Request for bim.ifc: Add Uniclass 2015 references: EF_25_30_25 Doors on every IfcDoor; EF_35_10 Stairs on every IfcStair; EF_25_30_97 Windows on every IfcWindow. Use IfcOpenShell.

First a look at what the model holds.

```python
import ifcopenshell

model = ifcopenshell.open("bim.ifc")
print(model.schema)
print("classifications:", [c.Name for c in model.by_type("IfcClassification")])
for ifc_class in ("IfcDoor", "IfcRoof", "IfcStair", "IfcWall", "IfcWindow"):
    print(ifc_class, len(model.by_type(ifc_class)))
```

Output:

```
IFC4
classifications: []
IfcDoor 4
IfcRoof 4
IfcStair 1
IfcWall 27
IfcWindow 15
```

```python
import ifcopenshell
import ifcopenshell.api.classification

model = ifcopenshell.open("bim.ifc")

system = ifcopenshell.api.classification.add_classification(model, classification="Uniclass 2015")

codes = {
    "IfcDoor": ("EF_25_30_25", "Doors"),
    "IfcStair": ("EF_35_10", "Stairs"),
    "IfcWindow": ("EF_25_30_97", "Windows"),
}
for ifc_class, (code, name) in codes.items():
    products = model.by_type(ifc_class)
    ifcopenshell.api.classification.add_reference(
        model, products=products, classification=system, identification=code, name=name
    )
    print(code, len(products))

model.write("bim_edited.ifc")
```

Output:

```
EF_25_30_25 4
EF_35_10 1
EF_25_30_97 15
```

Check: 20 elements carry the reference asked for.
